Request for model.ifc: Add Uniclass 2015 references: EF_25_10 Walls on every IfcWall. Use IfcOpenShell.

First a look at what the model holds.

```python
import ifcopenshell

model = ifcopenshell.open("model.ifc")
print(model.schema)
print("classifications:", [c.Name for c in model.by_type("IfcClassification")])
for ifc_class in ("IfcDoor", "IfcRoof", "IfcStair", "IfcWall", "IfcWindow"):
    print(ifc_class, len(model.by_type(ifc_class)))
```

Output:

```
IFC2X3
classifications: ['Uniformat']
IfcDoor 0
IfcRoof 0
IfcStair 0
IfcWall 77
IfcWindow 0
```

```python
import ifcopenshell
import ifcopenshell.api.classification

model = ifcopenshell.open("model.ifc")

# IFC2X3 requires Source and Edition and has no link from the project to the system.
system = model.create_entity("IfcClassification", Source="NBS", Edition="2015", Name="Uniclass 2015")

codes = {
    "IfcWall": ("EF_25_10", "Walls"),
}
for ifc_class, (code, name) in codes.items():
    products = model.by_type(ifc_class)
    ifcopenshell.api.classification.add_reference(
        model, products=products, classification=system, identification=code, name=name
    )
    print(code, len(products))

model.write("model_rev.ifc")
```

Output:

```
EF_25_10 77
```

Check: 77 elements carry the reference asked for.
